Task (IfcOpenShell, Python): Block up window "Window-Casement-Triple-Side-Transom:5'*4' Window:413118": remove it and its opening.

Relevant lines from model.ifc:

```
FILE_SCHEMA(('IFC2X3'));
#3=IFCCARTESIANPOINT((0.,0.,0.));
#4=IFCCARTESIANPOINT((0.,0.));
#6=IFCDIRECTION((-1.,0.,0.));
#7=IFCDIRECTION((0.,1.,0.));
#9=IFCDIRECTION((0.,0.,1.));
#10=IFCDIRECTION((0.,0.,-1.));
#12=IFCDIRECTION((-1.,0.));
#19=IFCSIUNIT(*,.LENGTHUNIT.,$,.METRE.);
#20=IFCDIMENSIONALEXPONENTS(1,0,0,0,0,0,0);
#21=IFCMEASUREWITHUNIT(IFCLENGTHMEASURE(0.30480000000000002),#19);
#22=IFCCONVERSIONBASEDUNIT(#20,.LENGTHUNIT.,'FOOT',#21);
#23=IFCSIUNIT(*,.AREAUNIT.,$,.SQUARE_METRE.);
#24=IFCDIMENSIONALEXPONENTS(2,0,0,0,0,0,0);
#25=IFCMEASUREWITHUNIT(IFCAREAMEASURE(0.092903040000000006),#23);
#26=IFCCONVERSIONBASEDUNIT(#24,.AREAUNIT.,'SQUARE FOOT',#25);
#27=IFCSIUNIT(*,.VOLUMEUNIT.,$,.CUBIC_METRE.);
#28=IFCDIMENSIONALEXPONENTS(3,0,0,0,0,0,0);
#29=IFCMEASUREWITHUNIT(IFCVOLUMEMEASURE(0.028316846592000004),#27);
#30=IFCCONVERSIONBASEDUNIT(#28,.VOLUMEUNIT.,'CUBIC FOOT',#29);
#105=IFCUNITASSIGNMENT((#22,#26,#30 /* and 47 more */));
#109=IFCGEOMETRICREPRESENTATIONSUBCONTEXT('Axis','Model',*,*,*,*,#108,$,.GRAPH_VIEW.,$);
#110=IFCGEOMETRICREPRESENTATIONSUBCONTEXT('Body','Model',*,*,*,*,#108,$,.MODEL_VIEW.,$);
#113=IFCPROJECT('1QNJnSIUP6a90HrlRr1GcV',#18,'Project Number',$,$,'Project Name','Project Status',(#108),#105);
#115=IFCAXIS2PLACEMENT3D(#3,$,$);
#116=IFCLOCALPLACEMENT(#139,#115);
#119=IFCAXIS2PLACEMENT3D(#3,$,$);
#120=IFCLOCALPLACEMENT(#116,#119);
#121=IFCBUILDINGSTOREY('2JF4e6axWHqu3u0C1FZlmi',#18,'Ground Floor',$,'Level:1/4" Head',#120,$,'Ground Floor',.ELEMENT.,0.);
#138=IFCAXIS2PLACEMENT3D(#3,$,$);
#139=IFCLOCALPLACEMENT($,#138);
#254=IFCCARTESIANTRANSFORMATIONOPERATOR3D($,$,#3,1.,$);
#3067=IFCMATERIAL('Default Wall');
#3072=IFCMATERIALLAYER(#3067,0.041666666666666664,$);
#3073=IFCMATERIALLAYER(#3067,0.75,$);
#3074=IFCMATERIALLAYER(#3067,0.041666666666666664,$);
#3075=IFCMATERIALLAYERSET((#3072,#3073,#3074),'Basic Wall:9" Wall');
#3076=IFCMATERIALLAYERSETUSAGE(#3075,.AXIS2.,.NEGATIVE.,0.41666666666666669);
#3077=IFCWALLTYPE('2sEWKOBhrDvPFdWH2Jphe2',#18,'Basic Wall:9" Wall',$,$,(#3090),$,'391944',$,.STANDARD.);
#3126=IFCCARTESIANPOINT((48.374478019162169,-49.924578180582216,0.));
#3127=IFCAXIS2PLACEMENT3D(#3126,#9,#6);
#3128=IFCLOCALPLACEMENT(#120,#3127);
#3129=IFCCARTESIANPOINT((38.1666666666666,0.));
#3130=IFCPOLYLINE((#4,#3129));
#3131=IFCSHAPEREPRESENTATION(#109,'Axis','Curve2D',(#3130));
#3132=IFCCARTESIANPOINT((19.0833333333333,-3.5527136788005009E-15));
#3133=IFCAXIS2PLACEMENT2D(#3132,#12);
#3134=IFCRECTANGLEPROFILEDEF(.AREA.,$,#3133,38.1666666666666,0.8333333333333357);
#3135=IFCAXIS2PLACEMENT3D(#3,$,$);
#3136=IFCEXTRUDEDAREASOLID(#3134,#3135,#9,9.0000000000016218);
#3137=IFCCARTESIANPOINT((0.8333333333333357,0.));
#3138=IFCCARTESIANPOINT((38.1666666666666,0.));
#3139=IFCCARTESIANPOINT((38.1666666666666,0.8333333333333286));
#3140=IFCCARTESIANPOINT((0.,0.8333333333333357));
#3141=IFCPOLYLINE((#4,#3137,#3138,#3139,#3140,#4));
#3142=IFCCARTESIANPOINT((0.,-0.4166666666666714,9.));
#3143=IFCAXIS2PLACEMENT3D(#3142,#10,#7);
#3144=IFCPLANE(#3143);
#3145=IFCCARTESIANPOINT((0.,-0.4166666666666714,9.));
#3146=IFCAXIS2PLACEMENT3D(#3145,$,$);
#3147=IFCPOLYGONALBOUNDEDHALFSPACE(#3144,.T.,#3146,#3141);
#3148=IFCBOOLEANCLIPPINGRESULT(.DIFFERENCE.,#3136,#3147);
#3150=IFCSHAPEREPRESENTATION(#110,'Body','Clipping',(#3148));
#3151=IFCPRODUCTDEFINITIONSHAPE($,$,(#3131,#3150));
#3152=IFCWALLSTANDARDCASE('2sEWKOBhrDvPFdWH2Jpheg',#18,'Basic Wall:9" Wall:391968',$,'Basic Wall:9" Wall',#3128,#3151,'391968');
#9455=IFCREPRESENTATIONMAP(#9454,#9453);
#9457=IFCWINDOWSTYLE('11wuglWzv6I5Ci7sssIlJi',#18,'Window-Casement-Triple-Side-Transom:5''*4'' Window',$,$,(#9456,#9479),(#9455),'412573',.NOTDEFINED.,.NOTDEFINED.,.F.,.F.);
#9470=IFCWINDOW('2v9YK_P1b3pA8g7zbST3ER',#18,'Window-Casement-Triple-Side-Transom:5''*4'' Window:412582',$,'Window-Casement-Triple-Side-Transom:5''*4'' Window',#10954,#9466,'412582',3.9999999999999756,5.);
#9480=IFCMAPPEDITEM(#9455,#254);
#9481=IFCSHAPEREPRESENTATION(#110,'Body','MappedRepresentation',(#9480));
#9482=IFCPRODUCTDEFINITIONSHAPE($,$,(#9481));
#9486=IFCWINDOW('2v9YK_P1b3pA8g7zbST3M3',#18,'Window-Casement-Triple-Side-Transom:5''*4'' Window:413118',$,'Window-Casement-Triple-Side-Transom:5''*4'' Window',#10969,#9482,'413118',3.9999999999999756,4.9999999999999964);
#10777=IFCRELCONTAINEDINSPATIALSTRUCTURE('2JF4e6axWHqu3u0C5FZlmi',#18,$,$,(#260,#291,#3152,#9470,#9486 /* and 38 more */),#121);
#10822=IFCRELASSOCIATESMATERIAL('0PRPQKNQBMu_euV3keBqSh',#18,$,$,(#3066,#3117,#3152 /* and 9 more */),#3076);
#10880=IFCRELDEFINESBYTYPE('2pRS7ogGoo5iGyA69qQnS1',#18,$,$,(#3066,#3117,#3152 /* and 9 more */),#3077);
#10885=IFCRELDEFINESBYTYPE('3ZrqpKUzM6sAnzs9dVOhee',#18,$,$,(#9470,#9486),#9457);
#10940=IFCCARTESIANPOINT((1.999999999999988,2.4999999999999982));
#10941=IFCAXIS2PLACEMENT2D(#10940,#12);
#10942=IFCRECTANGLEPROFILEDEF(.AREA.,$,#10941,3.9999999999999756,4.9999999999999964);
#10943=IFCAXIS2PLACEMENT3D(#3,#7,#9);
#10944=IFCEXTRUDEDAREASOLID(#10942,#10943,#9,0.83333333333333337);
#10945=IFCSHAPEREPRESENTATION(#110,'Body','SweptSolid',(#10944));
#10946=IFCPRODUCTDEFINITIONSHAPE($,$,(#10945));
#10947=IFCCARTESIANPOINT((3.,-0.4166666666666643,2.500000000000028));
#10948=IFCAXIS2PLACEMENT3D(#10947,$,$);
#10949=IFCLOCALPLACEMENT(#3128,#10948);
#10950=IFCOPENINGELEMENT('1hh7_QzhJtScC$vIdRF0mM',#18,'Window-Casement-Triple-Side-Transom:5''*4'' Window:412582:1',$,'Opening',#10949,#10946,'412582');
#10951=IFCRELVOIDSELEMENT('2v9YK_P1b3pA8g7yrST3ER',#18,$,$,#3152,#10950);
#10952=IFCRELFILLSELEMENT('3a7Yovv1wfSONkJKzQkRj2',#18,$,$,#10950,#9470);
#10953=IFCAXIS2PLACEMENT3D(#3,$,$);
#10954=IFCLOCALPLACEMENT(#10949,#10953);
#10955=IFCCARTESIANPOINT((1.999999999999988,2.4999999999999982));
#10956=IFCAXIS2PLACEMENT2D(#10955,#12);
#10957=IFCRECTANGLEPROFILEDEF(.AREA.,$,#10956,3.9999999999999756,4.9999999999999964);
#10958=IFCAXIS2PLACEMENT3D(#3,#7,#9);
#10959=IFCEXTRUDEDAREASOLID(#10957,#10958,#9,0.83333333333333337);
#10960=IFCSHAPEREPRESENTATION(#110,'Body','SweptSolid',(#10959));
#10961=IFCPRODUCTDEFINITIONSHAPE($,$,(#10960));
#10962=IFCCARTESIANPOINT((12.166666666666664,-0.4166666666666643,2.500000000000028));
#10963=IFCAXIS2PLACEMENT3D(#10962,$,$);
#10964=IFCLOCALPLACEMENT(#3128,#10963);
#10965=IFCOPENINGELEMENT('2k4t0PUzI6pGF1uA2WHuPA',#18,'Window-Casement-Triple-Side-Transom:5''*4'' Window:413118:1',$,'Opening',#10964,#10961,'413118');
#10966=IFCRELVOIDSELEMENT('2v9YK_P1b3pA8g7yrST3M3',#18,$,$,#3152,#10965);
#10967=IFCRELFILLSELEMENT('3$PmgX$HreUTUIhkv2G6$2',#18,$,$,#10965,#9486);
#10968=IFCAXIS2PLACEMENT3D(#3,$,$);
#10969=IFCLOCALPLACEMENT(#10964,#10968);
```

```python
import ifcopenshell
import ifcopenshell.api.feature
import ifcopenshell.api.root
import ifcopenshell.geom
import ifcopenshell.util.shape

model = ifcopenshell.open("model.ifc")
settings = ifcopenshell.geom.settings()


def volume(element):
    """Net volume in cubic metres, openings subtracted."""
    shape = ifcopenshell.geom.create_shape(settings, element)
    return ifcopenshell.util.shape.get_volume(shape.geometry)


window = model.by_id(9486)
opening = window.FillsVoids[0].RelatingOpeningElement
wall = opening.VoidsElements[0].RelatingBuildingElement
before = volume(wall)

ifcopenshell.api.root.remove_product(model, product=window)
ifcopenshell.api.feature.remove_feature(model, feature=opening)

after = volume(wall)

print(f"wall volume {before:.3f} -> {after:.3f} m3")

model.write("model_rev.ifc")
```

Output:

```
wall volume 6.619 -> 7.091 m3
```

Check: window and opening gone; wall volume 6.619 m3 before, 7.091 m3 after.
